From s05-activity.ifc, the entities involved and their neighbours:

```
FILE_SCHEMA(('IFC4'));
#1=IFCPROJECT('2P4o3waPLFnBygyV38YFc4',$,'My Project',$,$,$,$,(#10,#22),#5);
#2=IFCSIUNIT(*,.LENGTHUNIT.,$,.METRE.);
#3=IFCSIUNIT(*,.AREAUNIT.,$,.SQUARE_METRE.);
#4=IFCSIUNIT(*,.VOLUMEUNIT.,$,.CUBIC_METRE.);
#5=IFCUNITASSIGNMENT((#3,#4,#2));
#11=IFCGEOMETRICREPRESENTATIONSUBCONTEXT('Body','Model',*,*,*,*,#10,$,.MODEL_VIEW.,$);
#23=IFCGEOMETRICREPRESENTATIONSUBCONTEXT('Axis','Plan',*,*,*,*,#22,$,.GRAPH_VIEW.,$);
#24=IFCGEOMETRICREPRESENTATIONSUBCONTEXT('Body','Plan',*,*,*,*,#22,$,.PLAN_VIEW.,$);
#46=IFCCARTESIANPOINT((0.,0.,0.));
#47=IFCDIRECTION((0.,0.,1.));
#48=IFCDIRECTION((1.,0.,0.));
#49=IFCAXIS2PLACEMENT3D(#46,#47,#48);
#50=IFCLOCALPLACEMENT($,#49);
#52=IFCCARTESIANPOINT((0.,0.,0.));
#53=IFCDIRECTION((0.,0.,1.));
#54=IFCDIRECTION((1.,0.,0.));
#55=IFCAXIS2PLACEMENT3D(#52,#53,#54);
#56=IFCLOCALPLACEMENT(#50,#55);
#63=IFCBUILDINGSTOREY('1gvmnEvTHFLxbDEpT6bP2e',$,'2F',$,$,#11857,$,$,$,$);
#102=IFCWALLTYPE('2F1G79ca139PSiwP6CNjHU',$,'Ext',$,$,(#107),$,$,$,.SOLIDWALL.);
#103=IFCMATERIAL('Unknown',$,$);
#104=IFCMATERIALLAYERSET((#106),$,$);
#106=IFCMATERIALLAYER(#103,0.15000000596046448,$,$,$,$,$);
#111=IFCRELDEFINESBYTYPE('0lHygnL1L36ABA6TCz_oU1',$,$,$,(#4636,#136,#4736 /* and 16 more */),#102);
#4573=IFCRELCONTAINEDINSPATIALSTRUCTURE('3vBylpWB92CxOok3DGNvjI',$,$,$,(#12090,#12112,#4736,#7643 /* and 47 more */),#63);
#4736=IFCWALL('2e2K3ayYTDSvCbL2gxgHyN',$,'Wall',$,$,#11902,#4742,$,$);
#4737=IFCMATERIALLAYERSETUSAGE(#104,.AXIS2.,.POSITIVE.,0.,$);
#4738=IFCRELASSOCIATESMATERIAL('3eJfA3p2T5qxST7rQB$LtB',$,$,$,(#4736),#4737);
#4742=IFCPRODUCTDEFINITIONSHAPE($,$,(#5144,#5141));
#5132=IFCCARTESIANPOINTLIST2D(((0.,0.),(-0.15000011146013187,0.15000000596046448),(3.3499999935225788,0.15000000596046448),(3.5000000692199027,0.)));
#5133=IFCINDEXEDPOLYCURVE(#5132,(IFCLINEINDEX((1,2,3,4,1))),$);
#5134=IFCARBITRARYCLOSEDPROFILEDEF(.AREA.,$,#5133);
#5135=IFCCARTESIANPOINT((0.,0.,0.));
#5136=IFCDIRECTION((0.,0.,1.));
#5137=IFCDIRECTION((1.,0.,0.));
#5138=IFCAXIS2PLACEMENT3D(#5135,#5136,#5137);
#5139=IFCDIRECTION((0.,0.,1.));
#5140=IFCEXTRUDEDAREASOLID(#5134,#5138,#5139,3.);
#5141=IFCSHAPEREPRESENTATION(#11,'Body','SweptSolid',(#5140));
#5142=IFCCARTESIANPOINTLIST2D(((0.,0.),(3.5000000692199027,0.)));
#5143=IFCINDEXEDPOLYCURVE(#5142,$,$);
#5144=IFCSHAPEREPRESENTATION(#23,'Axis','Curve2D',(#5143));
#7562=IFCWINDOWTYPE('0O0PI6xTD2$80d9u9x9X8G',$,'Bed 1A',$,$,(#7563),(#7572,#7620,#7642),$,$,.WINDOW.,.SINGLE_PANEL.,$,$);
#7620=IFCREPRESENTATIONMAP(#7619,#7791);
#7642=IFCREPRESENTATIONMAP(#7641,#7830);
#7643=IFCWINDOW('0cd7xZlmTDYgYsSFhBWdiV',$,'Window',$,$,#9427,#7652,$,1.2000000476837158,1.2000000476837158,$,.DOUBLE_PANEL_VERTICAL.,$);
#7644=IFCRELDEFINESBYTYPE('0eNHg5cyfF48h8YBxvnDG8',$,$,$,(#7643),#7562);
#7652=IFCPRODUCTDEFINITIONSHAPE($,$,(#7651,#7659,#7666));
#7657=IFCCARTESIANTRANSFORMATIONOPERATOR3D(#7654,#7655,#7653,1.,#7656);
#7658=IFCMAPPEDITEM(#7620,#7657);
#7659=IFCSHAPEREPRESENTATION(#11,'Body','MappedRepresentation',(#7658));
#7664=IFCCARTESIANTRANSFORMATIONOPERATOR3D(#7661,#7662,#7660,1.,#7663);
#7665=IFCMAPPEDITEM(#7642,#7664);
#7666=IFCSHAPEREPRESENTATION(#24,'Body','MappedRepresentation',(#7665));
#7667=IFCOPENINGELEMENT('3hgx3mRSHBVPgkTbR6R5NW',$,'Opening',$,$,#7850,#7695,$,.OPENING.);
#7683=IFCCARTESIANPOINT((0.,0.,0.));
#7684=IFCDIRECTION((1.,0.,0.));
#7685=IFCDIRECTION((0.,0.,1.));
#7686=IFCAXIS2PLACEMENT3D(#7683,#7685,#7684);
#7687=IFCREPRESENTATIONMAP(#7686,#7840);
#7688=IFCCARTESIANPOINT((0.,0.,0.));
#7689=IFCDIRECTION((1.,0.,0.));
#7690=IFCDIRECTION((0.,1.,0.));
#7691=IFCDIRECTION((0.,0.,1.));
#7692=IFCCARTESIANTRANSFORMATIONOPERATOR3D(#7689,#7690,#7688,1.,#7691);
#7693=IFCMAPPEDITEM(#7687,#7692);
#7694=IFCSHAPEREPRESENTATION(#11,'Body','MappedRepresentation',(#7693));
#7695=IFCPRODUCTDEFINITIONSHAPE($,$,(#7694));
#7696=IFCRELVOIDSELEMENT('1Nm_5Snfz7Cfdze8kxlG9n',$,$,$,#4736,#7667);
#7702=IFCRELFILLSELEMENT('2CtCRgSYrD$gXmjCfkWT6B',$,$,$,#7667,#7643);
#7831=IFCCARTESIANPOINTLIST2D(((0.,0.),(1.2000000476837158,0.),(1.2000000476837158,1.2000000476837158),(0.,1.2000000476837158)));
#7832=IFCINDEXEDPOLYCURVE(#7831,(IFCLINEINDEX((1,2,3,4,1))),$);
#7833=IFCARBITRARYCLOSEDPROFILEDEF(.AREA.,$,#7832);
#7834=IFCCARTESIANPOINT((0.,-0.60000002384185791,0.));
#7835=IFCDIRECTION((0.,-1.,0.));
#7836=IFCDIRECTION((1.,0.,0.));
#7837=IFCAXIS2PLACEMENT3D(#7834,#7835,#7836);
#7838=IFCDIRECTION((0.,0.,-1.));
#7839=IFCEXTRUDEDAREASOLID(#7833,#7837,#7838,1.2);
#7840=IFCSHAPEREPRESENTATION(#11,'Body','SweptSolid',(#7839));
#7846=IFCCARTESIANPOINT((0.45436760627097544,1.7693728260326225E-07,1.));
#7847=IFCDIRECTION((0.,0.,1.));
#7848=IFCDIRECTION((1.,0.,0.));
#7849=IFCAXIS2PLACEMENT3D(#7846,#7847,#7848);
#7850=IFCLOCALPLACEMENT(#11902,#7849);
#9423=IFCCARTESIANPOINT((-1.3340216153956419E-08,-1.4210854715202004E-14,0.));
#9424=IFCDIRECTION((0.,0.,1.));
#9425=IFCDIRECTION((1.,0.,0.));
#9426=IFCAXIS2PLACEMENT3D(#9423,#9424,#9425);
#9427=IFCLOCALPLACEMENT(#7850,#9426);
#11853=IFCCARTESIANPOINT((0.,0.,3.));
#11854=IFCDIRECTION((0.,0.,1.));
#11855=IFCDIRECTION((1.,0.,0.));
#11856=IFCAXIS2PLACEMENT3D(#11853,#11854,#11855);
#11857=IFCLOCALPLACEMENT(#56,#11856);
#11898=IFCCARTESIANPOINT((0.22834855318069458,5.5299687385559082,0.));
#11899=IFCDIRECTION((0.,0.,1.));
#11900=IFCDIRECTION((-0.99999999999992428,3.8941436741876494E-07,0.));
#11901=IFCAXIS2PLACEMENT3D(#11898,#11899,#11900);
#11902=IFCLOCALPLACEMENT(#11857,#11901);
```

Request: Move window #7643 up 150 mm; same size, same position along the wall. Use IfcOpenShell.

```python
import numpy as np
import ifcopenshell
import ifcopenshell.api.geometry
import ifcopenshell.util.placement
import ifcopenshell.util.unit

model = ifcopenshell.open("s05-activity.ifc")
unit_scale = ifcopenshell.util.unit.calculate_unit_scale(model)

window = model.by_id(7643)
opening = window.FillsVoids[0].RelatingOpeningElement
dz = 0.15 / unit_scale

shift = np.array([0.0, 0.0, dz])
# The window is placed relative to its opening, so it follows when the opening moves.
matrix = ifcopenshell.util.placement.get_local_placement(opening.ObjectPlacement)
matrix[:3, 3] += shift
ifcopenshell.api.geometry.edit_object_placement(
    model, product=opening, matrix=matrix, is_si=False, should_transform_children=True
)

print(f"moved by {dz * unit_scale:+.3f} m")

model.write("s05-activity_rev.ifc")
```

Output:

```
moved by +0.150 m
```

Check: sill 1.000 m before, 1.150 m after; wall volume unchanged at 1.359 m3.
